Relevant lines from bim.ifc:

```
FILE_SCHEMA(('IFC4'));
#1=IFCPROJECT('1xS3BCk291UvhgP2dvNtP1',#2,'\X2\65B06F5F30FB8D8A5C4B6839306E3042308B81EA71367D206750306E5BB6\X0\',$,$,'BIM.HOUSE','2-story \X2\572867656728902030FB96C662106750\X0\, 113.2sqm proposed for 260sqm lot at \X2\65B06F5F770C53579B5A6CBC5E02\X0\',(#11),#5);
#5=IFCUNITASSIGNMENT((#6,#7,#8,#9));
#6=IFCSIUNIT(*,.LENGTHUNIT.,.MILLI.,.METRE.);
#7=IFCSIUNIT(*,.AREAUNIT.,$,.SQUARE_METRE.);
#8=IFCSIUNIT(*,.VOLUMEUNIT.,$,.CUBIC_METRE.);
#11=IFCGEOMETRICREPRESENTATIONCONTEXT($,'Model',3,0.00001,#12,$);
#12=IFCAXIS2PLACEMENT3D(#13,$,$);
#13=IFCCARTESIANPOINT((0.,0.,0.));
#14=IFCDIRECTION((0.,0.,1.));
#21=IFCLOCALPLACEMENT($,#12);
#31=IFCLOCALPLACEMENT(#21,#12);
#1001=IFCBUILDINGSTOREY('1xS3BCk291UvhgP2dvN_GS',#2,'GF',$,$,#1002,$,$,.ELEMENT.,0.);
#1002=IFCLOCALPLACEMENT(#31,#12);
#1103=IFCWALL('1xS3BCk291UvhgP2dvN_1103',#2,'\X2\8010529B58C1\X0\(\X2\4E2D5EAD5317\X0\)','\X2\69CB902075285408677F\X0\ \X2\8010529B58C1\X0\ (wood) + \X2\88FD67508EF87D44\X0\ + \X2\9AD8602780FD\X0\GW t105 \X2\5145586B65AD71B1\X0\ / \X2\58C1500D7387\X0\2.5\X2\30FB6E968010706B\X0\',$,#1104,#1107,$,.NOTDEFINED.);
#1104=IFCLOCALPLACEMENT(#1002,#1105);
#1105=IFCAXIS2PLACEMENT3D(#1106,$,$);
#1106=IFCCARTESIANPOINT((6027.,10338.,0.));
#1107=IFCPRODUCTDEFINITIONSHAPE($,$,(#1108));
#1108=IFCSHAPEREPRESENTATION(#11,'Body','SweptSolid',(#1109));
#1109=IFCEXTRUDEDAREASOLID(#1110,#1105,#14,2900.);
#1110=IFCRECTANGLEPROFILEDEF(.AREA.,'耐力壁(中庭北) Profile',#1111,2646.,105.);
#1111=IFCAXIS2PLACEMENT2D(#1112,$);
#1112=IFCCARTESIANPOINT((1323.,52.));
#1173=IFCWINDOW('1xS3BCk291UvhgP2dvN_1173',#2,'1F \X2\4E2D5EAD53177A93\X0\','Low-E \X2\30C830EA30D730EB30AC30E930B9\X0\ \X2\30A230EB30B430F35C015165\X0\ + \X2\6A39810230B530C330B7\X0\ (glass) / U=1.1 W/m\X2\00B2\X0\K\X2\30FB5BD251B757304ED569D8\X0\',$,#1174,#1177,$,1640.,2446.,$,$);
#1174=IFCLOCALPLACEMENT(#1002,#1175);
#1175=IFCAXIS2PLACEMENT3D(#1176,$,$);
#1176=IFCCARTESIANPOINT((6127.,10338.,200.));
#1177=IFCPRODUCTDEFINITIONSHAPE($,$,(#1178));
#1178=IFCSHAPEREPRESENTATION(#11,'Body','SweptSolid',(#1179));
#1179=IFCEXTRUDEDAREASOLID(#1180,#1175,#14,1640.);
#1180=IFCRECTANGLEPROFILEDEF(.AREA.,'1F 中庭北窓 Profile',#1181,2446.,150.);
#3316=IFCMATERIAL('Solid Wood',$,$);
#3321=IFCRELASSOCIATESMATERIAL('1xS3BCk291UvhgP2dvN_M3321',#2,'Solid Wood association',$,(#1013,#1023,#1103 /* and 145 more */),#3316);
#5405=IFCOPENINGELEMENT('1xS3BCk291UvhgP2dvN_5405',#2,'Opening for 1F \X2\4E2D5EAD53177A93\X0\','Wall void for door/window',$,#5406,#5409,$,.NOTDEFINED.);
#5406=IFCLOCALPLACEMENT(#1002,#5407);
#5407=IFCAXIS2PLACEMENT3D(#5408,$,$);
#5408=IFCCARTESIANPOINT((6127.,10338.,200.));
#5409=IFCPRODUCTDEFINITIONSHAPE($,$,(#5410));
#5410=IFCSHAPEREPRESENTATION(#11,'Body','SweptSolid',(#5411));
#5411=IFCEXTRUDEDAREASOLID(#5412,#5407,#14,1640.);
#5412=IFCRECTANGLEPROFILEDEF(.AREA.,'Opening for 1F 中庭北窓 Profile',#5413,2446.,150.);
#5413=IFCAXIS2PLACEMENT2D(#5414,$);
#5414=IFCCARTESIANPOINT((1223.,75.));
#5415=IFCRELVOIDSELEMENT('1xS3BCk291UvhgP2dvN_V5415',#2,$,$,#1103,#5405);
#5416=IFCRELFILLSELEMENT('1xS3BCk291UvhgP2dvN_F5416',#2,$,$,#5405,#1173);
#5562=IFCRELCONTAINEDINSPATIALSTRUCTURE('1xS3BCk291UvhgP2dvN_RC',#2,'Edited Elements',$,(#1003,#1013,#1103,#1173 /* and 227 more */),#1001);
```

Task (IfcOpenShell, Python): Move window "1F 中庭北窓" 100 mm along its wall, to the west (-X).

```python
import ifcopenshell
import ifcopenshell.api.geometry
import ifcopenshell.util.placement

model = ifcopenshell.open("bim.ifc")

window = model.by_id(1173)
opening = window.FillsVoids[0].RelatingOpeningElement
wall = opening.VoidsElements[0].RelatingBuildingElement

wall_matrix = ifcopenshell.util.placement.get_local_placement(wall.ObjectPlacement)
shift = wall_matrix[:3, 0] * -100.0
before = ifcopenshell.util.placement.get_local_placement(window.ObjectPlacement)[:3, 3].copy()

# The window is not placed relative to its opening, so move both.
for product in (opening, window):
    matrix = ifcopenshell.util.placement.get_local_placement(product.ObjectPlacement)
    matrix[:3, 3] += shift
    ifcopenshell.api.geometry.edit_object_placement(model, product=product, matrix=matrix, is_si=False)

after = ifcopenshell.util.placement.get_local_placement(window.ObjectPlacement)[:3, 3]
print("window moved by", (after - before).round(3) + 0.0)

model.write("bim_edited.ifc")
```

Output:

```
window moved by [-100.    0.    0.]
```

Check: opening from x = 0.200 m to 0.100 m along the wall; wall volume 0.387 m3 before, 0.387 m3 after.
